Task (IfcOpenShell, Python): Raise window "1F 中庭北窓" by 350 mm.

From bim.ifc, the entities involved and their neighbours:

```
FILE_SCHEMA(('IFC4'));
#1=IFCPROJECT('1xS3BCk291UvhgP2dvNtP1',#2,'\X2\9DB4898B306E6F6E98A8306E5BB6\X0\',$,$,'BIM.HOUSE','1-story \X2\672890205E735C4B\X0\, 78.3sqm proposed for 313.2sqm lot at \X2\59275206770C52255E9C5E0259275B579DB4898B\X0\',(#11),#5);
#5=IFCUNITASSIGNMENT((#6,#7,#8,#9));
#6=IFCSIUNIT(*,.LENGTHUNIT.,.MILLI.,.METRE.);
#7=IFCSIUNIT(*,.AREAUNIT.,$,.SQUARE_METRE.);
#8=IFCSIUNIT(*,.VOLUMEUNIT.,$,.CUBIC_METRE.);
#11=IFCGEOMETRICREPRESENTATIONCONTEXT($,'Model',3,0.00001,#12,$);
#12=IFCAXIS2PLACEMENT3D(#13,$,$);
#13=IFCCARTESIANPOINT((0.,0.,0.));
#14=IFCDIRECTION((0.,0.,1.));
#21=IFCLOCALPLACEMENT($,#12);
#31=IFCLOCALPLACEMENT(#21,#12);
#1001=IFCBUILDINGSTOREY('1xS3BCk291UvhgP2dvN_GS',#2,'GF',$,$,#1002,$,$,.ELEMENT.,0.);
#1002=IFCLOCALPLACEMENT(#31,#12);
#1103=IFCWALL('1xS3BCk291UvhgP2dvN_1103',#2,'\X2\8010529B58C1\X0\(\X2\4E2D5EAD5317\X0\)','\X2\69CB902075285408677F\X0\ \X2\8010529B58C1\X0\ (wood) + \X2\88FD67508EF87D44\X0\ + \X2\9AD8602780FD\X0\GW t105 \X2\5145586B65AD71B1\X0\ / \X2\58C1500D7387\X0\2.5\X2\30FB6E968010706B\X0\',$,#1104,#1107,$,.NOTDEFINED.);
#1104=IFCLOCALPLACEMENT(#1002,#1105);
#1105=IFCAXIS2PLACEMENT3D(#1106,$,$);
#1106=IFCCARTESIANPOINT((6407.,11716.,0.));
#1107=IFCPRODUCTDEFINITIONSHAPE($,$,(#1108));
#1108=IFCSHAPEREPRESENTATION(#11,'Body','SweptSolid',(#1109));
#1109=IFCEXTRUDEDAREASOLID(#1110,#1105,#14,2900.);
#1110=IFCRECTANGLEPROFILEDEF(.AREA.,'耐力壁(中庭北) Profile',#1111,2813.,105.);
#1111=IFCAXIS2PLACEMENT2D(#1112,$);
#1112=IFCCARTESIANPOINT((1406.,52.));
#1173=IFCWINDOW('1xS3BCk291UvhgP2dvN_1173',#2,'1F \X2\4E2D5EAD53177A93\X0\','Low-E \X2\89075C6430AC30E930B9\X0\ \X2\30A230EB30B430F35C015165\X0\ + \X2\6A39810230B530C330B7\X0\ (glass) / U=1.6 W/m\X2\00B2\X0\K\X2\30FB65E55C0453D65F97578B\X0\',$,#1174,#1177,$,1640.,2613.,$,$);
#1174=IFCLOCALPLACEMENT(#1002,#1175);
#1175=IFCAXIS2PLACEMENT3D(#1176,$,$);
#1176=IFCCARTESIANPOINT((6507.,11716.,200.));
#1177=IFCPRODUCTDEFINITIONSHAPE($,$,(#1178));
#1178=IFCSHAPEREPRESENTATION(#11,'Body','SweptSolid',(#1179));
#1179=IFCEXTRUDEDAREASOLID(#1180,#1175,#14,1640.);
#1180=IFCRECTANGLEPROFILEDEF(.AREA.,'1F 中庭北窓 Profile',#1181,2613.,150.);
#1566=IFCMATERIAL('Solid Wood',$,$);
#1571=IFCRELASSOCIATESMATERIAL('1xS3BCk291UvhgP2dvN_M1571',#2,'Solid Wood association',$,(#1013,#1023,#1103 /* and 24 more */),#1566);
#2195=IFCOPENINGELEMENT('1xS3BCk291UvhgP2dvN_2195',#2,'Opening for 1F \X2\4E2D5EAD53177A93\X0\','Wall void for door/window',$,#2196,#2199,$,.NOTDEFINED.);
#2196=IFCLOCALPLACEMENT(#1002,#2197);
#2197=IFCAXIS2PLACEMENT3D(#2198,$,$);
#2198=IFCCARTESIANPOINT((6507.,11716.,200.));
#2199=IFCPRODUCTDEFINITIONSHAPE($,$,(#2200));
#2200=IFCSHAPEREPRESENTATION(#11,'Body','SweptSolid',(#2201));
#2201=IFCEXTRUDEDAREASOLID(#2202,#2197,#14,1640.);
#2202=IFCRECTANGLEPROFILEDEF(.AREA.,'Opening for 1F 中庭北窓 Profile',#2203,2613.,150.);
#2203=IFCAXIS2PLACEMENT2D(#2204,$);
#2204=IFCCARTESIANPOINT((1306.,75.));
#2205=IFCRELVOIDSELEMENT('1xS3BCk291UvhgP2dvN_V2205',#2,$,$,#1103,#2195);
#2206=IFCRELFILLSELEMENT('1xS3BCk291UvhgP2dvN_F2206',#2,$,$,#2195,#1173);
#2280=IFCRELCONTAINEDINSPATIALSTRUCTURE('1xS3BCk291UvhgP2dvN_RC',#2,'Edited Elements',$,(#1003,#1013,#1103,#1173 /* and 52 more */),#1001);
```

```python
import numpy as np
import ifcopenshell
import ifcopenshell.api.geometry
import ifcopenshell.util.placement
import ifcopenshell.util.unit

model = ifcopenshell.open("bim.ifc")
unit_scale = ifcopenshell.util.unit.calculate_unit_scale(model)

window = model.by_guid("1xS3BCk291UvhgP2dvN_1173")
opening = window.FillsVoids[0].RelatingOpeningElement
dz = 0.35 / unit_scale

shift = np.array([0.0, 0.0, dz])
# The window is not placed relative to its opening, so move both.
for product in (opening, window):
    matrix = ifcopenshell.util.placement.get_local_placement(product.ObjectPlacement)
    matrix[:3, 3] += shift
    ifcopenshell.api.geometry.edit_object_placement(model, product=product, matrix=matrix, is_si=False)

print(f"moved by {dz * unit_scale:+.3f} m")

model.write("bim_rev.ifc")
```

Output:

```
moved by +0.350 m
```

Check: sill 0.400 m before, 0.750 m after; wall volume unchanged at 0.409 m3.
